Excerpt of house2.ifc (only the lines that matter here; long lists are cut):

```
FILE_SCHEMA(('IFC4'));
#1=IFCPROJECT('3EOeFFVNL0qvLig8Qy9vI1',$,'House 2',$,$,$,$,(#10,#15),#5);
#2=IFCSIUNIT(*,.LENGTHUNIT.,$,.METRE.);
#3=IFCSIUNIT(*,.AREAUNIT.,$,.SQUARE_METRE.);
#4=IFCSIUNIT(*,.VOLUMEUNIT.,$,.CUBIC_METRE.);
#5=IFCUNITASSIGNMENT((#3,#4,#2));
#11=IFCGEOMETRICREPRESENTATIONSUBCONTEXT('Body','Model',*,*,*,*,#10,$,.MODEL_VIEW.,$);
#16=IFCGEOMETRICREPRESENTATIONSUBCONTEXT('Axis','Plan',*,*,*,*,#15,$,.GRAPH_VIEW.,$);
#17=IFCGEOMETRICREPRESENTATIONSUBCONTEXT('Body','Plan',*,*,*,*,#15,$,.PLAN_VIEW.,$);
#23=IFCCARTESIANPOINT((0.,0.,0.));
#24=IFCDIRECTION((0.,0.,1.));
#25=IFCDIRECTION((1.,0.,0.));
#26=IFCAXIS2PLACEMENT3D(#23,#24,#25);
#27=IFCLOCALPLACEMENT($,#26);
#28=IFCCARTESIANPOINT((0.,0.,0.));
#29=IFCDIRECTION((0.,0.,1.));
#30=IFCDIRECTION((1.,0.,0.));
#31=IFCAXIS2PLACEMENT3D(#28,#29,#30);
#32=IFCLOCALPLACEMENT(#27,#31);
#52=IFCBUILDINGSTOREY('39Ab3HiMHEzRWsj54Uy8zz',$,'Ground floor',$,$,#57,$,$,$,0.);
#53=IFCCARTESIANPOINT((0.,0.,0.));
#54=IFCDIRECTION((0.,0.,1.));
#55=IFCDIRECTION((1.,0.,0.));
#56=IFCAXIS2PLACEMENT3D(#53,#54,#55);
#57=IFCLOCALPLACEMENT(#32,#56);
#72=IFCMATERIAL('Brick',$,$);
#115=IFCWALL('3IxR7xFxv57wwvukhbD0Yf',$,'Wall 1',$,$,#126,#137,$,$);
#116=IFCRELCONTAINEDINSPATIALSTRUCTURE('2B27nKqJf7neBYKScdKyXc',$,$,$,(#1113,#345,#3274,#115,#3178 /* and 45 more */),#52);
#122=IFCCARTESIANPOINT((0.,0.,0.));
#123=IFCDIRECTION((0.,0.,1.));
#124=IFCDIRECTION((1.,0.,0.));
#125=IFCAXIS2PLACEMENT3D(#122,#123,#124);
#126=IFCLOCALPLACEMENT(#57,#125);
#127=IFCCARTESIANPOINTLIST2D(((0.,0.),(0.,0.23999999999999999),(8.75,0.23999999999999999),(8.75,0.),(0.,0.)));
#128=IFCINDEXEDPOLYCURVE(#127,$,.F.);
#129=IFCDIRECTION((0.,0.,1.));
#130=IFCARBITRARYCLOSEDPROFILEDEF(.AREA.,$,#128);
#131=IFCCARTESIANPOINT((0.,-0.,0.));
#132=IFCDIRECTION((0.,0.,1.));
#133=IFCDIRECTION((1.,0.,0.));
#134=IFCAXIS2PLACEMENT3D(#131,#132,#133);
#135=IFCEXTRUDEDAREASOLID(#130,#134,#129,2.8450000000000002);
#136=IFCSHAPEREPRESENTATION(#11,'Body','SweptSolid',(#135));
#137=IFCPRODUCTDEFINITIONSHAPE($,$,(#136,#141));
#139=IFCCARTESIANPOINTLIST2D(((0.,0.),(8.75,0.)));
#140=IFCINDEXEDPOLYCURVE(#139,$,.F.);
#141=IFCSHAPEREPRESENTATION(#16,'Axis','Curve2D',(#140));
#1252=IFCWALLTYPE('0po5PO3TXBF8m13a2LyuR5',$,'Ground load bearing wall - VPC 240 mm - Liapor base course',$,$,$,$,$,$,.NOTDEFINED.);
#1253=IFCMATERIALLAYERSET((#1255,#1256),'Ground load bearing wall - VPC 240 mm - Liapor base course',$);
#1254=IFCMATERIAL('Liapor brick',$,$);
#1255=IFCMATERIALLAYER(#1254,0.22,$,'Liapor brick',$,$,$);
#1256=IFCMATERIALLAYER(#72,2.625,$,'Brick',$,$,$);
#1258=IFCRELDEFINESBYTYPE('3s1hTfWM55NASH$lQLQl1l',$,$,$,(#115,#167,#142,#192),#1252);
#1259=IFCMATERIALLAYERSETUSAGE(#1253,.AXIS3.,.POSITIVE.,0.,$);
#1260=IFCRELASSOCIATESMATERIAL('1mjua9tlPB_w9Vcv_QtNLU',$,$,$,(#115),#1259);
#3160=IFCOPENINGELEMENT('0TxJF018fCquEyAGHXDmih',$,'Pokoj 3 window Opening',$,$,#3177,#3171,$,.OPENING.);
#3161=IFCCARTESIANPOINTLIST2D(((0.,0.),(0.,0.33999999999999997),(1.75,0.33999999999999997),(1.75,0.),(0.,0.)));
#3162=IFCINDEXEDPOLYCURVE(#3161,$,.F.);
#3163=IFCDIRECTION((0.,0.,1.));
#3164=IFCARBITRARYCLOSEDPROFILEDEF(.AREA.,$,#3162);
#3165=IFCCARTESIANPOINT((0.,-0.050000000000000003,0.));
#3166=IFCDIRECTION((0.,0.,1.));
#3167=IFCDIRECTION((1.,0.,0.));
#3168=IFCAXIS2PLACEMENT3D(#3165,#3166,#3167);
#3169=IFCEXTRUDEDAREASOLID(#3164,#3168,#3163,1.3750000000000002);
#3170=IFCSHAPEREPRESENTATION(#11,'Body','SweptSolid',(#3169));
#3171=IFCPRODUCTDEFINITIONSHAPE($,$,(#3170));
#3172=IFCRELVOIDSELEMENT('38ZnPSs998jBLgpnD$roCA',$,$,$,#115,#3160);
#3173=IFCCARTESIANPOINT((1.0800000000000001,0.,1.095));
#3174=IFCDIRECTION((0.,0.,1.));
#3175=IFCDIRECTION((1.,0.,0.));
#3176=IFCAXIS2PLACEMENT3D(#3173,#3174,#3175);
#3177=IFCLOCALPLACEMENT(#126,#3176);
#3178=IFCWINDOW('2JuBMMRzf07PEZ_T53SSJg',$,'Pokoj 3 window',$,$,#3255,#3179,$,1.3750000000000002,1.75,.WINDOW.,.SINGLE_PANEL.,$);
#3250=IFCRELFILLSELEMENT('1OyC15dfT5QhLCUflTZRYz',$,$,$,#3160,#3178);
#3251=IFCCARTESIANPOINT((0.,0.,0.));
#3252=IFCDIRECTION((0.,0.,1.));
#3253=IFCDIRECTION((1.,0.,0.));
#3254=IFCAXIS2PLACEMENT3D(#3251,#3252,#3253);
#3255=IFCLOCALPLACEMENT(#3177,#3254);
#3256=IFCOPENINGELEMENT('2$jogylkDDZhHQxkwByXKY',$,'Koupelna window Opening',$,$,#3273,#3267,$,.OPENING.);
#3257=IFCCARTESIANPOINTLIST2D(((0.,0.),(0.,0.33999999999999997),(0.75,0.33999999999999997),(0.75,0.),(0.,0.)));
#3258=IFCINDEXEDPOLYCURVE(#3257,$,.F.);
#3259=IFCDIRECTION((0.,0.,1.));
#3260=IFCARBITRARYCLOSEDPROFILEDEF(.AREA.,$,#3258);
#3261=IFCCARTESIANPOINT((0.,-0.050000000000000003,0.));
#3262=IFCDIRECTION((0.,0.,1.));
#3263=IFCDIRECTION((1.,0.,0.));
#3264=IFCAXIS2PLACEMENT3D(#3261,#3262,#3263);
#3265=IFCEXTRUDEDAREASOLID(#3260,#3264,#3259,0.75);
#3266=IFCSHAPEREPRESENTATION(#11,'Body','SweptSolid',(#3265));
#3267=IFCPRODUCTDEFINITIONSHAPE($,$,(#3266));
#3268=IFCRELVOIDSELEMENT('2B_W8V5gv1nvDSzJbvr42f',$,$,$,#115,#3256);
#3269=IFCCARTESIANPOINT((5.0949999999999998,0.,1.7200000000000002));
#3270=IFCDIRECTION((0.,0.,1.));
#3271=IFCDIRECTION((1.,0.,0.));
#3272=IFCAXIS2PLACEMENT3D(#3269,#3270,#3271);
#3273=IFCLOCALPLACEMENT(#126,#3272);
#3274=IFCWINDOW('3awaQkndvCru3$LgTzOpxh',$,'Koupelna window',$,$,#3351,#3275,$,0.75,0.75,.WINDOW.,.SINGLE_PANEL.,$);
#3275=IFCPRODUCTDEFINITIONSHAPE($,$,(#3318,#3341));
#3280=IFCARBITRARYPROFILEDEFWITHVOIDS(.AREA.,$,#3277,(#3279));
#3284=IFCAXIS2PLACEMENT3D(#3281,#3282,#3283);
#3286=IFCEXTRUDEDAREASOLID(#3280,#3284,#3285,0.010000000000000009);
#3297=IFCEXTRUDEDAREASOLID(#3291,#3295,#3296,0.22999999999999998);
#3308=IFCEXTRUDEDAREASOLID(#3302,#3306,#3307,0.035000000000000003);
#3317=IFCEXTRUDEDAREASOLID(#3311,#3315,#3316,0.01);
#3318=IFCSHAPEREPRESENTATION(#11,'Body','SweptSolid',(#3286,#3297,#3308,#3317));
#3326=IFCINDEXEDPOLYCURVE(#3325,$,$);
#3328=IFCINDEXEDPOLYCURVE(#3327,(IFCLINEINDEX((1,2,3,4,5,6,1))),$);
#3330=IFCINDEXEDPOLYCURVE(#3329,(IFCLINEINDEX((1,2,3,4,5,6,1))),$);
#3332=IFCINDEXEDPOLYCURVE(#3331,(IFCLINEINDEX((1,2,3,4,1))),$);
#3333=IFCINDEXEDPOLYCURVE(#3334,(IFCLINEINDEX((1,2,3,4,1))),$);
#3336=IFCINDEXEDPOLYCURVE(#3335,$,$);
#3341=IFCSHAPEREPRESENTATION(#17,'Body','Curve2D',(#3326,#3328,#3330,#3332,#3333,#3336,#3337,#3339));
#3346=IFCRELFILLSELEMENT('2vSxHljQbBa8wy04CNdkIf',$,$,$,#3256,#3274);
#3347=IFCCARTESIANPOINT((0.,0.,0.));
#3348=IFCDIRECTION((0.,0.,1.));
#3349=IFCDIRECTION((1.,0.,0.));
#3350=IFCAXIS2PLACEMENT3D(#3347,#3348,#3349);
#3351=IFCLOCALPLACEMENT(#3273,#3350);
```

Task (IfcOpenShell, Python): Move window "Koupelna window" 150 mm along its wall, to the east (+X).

```python
import ifcopenshell
import ifcopenshell.api.geometry
import ifcopenshell.util.placement

model = ifcopenshell.open("house2.ifc")

window = model.by_guid("3awaQkndvCru3$LgTzOpxh")
opening = window.FillsVoids[0].RelatingOpeningElement
wall = opening.VoidsElements[0].RelatingBuildingElement

wall_matrix = ifcopenshell.util.placement.get_local_placement(wall.ObjectPlacement)
shift = wall_matrix[:3, 0] * 0.15
before = ifcopenshell.util.placement.get_local_placement(window.ObjectPlacement)[:3, 3].copy()

# The window is placed relative to its opening, so it follows when the opening moves.
matrix = ifcopenshell.util.placement.get_local_placement(opening.ObjectPlacement)
matrix[:3, 3] += shift
ifcopenshell.api.geometry.edit_object_placement(
    model, product=opening, matrix=matrix, is_si=False, should_transform_children=True
)

after = ifcopenshell.util.placement.get_local_placement(window.ObjectPlacement)[:3, 3]
print("window moved by", (after - before).round(3) + 0.0)

model.write("house2-out.ifc")
```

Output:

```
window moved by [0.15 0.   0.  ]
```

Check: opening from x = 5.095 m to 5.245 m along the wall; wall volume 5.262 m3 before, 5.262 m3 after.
